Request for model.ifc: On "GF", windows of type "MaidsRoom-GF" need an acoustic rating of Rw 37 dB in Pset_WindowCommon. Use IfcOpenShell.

First a look at what the model holds.

```python
import ifcopenshell
import ifcopenshell.util.element

model = ifcopenshell.open("model.ifc")
print(model.schema)
storey = next(s for s in model.by_type("IfcBuildingStorey") if s.Name == "GF")
windows = [e for e in ifcopenshell.util.element.get_decomposition(storey) if e.is_a("IfcWindow")]
seen = {}
for e in windows:
    element_type = ifcopenshell.util.element.get_type(e)
    key = (element_type.Name if element_type != e and element_type else None, ifcopenshell.util.element.get_pset(e, "Pset_WindowCommon", "AcousticRating"))
    seen[key] = seen.get(key, 0) + 1
for (name, value), count in sorted(seen.items(), key=str):
    print(count, "x", name, "|", value)
```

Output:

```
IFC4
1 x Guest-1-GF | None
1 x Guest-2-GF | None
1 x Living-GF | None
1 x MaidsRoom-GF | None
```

```python
import ifcopenshell
import ifcopenshell.api.pset
import ifcopenshell.util.element

model = ifcopenshell.open("model.ifc")

storey = next(s for s in model.by_type("IfcBuildingStorey") if s.Name == "GF")
windows = [e for e in ifcopenshell.util.element.get_decomposition(storey) if e.is_a("IfcWindow")]

count = 0
for e in windows:
    element_type = ifcopenshell.util.element.get_type(e)
    if element_type in (None, e) or element_type.Name != "MaidsRoom-GF":
        continue
    # add_pset returns the element's existing set when there is one.
    pset = ifcopenshell.api.pset.add_pset(model, product=e, name="Pset_WindowCommon")
    ifcopenshell.api.pset.edit_pset(model, pset=pset, properties={"AcousticRating": "Rw 37 dB"})
    count += 1

print(count, "windows updated")

model.write("model-out.ifc")
```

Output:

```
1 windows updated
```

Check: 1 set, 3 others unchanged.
